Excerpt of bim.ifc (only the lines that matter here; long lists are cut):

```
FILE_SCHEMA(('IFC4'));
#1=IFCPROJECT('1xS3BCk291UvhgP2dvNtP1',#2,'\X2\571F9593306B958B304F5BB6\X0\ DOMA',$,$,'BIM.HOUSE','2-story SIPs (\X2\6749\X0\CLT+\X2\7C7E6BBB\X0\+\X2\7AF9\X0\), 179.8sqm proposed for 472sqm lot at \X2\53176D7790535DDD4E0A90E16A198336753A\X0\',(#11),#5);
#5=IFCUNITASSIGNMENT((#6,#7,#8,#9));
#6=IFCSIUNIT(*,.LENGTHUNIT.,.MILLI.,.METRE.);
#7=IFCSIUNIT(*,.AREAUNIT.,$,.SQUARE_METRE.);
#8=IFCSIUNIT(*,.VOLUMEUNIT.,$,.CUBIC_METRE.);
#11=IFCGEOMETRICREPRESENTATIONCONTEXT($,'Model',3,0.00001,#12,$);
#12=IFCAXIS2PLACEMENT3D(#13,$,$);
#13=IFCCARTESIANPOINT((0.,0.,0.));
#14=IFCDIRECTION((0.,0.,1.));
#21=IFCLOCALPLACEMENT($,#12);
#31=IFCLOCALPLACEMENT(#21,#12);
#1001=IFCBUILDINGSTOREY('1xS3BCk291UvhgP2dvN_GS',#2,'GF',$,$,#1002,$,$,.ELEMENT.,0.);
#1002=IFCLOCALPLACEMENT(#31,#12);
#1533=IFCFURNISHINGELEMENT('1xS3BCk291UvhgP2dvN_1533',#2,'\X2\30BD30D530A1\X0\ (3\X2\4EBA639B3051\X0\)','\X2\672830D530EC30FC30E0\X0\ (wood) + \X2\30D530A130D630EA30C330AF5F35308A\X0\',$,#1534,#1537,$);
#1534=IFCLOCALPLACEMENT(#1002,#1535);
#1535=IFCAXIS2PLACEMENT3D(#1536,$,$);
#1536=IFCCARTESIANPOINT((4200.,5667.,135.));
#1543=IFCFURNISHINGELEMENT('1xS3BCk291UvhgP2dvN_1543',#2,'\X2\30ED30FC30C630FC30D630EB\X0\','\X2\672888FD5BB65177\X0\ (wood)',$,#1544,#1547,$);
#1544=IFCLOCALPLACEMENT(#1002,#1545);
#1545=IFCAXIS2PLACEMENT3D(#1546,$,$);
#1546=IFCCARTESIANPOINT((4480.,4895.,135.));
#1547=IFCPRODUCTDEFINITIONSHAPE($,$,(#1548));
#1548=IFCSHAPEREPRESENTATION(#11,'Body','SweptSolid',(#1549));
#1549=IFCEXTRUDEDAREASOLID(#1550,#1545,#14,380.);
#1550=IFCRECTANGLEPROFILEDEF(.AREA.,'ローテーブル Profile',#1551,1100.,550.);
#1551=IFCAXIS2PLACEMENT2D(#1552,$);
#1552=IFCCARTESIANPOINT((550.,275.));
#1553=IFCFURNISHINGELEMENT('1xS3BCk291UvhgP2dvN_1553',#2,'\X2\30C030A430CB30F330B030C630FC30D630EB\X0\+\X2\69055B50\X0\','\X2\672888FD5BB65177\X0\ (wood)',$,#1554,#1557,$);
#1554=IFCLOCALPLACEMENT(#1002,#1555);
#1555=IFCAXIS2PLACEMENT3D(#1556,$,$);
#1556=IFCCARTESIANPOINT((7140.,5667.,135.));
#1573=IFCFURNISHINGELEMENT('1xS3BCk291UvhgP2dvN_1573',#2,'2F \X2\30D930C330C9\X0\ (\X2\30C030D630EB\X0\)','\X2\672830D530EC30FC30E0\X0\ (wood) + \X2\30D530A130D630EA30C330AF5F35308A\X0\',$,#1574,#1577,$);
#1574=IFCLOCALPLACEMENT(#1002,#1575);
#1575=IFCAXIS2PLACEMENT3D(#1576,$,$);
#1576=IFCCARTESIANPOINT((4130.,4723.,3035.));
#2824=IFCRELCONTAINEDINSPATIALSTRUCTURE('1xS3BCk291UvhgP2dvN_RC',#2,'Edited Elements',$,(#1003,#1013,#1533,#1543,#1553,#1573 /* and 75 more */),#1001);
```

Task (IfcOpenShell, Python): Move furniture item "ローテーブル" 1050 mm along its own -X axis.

```python
import ifcopenshell
import ifcopenshell.api.geometry
import ifcopenshell.util.placement

model = ifcopenshell.open("bim.ifc")

item = model.by_guid("1xS3BCk291UvhgP2dvN_1543")
matrix = ifcopenshell.util.placement.get_local_placement(item.ObjectPlacement)
matrix[:3, 3] -= matrix[:3, 0] * 1050.0
ifcopenshell.api.geometry.edit_object_placement(model, product=item, matrix=matrix, is_si=False)

print(ifcopenshell.util.placement.get_local_placement(item.ObjectPlacement).round(3) + 0.0)

model.write("bim_v2.ifc")
```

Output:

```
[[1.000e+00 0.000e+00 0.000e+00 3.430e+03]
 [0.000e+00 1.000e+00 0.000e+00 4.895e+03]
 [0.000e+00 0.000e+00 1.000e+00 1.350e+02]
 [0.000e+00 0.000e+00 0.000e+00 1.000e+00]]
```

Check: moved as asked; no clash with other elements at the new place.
